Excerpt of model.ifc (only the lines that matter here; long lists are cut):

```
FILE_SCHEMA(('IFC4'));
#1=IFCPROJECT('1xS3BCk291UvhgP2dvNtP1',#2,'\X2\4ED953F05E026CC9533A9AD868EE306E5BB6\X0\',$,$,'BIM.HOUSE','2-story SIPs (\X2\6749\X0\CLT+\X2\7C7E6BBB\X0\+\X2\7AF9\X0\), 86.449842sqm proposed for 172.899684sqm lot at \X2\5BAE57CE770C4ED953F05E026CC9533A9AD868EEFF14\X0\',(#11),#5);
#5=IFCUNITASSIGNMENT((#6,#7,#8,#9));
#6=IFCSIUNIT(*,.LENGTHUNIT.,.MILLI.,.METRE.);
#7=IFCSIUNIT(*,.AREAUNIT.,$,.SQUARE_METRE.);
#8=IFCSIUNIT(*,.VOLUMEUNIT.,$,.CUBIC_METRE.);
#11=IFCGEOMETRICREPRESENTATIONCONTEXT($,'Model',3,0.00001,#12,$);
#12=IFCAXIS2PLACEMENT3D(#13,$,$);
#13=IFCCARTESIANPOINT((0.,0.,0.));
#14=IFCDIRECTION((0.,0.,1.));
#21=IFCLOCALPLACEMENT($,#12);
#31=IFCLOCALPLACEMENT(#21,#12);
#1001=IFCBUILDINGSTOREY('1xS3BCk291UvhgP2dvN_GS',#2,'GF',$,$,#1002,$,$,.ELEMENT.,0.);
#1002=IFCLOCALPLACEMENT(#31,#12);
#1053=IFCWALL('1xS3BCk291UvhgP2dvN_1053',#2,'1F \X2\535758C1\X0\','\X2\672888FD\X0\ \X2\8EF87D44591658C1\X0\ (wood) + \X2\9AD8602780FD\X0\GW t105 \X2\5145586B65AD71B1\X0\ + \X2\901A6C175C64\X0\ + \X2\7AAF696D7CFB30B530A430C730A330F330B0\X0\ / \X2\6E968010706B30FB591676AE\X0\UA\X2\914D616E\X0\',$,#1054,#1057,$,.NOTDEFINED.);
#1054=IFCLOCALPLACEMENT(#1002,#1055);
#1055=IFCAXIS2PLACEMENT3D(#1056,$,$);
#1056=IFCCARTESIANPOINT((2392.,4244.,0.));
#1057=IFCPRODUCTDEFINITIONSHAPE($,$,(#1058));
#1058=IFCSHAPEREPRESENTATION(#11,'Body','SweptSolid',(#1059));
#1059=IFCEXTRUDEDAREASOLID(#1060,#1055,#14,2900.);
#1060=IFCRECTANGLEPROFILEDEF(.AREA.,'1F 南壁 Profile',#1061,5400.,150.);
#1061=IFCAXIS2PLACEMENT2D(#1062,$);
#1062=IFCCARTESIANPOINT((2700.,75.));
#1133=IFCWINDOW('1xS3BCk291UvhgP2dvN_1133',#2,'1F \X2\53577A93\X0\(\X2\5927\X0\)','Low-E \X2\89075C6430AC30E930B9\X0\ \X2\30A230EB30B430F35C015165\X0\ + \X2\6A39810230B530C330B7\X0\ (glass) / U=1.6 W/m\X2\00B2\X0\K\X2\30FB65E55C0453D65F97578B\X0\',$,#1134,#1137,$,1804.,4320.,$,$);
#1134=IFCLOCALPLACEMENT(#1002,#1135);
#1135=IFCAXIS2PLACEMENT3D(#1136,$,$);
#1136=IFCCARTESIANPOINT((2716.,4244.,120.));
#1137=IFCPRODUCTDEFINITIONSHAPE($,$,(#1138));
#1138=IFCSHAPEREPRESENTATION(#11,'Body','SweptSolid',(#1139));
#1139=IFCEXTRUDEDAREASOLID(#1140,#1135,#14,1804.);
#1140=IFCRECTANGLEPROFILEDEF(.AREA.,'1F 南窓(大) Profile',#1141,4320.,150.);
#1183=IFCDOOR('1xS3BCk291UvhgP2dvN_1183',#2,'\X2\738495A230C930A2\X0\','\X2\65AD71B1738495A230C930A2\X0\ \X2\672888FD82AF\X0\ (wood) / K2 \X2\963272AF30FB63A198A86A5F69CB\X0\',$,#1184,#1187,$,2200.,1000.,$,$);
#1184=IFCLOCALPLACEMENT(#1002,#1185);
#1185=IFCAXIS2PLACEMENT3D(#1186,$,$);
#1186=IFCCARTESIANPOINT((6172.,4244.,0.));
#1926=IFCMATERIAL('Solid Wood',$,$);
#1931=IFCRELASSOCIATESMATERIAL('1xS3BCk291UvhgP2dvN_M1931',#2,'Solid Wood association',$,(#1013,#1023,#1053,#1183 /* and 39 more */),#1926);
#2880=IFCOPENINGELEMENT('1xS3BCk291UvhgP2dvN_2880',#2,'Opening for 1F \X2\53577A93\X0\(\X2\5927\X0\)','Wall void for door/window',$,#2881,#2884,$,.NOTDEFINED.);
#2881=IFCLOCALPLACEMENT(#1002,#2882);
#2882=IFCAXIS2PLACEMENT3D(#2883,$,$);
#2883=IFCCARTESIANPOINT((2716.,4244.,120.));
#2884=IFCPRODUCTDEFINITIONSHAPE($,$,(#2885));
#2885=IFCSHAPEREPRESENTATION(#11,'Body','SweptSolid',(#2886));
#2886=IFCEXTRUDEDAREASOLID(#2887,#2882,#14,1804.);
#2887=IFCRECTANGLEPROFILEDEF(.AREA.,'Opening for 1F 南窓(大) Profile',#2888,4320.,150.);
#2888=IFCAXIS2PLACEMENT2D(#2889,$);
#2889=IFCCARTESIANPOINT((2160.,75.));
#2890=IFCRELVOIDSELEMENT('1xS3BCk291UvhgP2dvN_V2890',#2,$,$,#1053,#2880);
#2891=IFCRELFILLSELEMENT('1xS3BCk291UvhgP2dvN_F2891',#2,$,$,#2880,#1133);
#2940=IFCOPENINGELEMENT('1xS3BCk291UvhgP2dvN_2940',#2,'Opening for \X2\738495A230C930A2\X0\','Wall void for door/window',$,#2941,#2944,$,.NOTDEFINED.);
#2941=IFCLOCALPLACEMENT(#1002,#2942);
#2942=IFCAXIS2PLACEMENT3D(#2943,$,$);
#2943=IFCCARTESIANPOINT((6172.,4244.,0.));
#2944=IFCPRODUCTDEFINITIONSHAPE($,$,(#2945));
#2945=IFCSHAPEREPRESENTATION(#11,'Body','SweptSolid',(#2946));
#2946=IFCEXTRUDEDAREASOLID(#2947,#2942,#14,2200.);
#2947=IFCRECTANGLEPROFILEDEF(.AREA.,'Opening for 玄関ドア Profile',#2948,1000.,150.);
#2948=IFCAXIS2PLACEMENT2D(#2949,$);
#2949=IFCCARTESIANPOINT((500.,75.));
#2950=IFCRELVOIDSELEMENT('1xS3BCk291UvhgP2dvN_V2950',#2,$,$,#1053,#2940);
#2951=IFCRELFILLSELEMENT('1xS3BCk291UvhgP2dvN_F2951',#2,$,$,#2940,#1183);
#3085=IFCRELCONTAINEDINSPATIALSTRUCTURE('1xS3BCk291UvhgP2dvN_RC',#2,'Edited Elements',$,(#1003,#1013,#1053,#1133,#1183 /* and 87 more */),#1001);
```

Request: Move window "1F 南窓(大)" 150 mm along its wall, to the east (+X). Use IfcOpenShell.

```python
import ifcopenshell
import ifcopenshell.api.geometry
import ifcopenshell.util.placement
import ifcopenshell.util.unit

model = ifcopenshell.open("model.ifc")
unit_scale = ifcopenshell.util.unit.calculate_unit_scale(model)

window = model.by_guid("1xS3BCk291UvhgP2dvN_1133")
opening = window.FillsVoids[0].RelatingOpeningElement
wall = opening.VoidsElements[0].RelatingBuildingElement

wall_matrix = ifcopenshell.util.placement.get_local_placement(wall.ObjectPlacement)
shift = wall_matrix[:3, 0] * 0.15 / unit_scale
before = ifcopenshell.util.placement.get_local_placement(window.ObjectPlacement)[:3, 3].copy()

# The window is not placed relative to its opening, so move both.
for product in (opening, window):
    matrix = ifcopenshell.util.placement.get_local_placement(product.ObjectPlacement)
    matrix[:3, 3] += shift
    ifcopenshell.api.geometry.edit_object_placement(model, product=product, matrix=matrix, is_si=False)

after = ifcopenshell.util.placement.get_local_placement(window.ObjectPlacement)[:3, 3]
print("window moved by", (after - before).round(3) + 0.0)

model.write("model_edited.ifc")
```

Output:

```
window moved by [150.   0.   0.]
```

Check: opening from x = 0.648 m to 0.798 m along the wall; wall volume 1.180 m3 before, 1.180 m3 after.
